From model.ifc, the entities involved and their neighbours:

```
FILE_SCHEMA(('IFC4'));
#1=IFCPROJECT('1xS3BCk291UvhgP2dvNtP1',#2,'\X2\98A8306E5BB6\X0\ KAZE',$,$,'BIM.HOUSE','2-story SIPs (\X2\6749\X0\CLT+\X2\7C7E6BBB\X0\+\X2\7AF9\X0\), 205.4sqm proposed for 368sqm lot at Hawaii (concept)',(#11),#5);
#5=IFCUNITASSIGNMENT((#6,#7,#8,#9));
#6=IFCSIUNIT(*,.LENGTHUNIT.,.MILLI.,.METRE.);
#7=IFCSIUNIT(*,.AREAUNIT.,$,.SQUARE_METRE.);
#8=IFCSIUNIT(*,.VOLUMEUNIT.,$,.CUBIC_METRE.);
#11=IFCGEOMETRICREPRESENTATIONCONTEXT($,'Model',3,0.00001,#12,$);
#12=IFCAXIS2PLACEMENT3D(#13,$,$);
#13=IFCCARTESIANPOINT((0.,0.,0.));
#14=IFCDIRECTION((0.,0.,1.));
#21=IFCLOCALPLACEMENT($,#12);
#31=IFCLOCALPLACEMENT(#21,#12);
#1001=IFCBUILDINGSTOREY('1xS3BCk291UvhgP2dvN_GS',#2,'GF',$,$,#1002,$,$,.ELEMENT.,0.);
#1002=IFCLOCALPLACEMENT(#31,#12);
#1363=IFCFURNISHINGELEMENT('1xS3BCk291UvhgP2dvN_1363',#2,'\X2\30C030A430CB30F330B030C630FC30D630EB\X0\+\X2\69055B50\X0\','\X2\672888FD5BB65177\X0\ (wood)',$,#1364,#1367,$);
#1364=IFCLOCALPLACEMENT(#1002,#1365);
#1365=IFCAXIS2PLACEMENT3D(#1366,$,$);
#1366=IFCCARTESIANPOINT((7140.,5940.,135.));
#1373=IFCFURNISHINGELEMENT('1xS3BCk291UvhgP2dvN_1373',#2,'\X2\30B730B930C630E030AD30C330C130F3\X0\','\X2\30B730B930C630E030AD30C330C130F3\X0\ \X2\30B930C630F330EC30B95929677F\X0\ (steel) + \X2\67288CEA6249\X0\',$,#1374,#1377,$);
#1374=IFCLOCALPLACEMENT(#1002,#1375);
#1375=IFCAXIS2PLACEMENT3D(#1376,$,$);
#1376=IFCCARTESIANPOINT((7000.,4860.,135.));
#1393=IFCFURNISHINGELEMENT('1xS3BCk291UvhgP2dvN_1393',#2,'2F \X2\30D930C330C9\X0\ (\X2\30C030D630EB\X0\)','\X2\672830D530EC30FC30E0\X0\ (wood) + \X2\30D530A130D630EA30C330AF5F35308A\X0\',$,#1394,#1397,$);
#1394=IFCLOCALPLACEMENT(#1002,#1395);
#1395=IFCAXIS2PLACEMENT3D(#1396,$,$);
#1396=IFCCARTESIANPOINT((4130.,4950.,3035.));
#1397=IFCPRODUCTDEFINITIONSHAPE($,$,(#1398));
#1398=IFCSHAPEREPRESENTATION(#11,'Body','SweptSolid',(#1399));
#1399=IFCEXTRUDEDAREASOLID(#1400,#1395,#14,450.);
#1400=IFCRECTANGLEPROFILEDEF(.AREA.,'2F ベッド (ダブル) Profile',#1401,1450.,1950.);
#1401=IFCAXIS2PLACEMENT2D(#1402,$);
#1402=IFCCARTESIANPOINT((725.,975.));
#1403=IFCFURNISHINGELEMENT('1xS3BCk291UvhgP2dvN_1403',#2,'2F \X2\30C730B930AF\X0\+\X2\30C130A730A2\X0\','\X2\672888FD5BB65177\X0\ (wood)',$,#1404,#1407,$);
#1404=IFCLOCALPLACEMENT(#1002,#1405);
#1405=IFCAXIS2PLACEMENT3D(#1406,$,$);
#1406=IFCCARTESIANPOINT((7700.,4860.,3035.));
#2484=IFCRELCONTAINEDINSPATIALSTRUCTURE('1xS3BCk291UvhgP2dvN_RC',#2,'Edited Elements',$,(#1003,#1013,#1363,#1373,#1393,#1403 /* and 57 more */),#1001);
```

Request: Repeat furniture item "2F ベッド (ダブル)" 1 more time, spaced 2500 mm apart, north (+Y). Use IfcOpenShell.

```python
import numpy as np
import ifcopenshell
import ifcopenshell.api.geometry
import ifcopenshell.api.root
import ifcopenshell.util.element
import ifcopenshell.util.placement
import ifcopenshell.util.unit

model = ifcopenshell.open("model.ifc")
unit_scale = ifcopenshell.util.unit.calculate_unit_scale(model)


def reuse_history(source, copy):
    """copy_class also copies each property set's owner history, people and application; keep the originals."""
    for rel in copy.IsDefinedBy:
        if rel.is_a("IfcRelDefinesByProperties") and (history := rel.RelatingPropertyDefinition.OwnerHistory):
            rel.RelatingPropertyDefinition.OwnerHistory = source.OwnerHistory
            ifcopenshell.util.element.remove_deep2(model, history)


source = model.by_id(1393)
base = ifcopenshell.util.placement.get_local_placement(source.ObjectPlacement)
step = np.array([0.0, 1.0, 0.0]) * 2.5 / unit_scale

for i in range(1, 2):
    copy = ifcopenshell.api.root.copy_class(model, product=source)
    copy.Representation = ifcopenshell.util.element.copy_deep(
        model, source.Representation, exclude=["IfcGeometricRepresentationContext", "IfcRepresentationMap"]
    )
    reuse_history(source, copy)
    matrix = base.copy()
    matrix[:3, 3] += i * step
    print("added at", matrix[:3, 3].round(3) + 0.0)
    ifcopenshell.api.geometry.edit_object_placement(model, product=copy, matrix=matrix, is_si=False)

model.write("model_v2.ifc")
```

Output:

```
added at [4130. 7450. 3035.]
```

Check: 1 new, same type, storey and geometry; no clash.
